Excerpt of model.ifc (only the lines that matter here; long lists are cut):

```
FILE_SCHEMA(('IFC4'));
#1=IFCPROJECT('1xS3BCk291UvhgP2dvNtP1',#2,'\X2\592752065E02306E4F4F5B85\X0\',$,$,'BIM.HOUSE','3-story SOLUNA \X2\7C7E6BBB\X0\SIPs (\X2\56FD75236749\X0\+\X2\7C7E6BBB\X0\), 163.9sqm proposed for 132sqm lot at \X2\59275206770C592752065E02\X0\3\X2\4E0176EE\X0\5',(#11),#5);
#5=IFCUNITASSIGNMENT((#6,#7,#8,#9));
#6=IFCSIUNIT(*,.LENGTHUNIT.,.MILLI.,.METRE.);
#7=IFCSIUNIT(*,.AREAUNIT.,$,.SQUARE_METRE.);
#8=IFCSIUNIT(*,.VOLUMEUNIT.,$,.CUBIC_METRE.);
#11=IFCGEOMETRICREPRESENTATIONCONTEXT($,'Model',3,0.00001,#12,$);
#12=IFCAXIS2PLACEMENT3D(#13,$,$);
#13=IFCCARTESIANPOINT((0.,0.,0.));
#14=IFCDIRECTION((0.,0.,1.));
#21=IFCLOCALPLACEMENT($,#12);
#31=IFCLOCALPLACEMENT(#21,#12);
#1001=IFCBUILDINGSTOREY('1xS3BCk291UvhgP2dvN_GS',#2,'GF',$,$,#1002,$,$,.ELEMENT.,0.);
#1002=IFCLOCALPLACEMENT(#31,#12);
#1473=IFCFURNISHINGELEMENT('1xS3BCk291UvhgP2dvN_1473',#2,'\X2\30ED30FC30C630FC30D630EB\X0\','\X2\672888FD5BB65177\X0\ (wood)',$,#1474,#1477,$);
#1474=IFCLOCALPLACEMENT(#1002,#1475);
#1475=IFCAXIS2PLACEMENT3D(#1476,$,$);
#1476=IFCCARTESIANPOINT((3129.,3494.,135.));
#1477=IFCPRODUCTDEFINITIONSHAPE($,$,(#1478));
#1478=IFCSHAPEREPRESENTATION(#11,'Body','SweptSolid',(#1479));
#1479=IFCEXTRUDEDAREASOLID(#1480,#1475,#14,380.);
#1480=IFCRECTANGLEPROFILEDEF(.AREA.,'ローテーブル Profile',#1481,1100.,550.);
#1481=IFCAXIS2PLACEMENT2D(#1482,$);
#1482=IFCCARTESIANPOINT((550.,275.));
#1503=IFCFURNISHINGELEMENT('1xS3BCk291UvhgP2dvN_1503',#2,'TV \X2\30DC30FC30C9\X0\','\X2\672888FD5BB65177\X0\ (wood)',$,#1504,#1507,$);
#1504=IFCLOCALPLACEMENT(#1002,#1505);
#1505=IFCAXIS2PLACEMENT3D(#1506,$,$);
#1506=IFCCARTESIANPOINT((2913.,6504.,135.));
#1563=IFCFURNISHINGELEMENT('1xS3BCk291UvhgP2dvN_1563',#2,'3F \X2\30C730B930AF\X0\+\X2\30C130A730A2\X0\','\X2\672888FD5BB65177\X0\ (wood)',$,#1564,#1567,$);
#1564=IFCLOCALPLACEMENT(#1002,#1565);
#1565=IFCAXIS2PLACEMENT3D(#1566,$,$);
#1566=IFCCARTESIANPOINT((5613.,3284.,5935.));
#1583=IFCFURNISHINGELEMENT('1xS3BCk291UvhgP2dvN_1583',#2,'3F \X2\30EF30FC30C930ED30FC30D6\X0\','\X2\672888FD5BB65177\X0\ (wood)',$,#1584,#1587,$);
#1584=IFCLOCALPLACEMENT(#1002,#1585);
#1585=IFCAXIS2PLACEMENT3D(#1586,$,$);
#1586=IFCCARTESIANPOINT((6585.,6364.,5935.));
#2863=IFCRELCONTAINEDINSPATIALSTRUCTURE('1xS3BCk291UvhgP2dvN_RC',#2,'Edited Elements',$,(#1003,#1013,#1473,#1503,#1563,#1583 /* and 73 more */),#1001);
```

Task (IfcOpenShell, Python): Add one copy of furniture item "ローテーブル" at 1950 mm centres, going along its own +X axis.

```python
import ifcopenshell
import ifcopenshell.api.geometry
import ifcopenshell.api.root
import ifcopenshell.util.element
import ifcopenshell.util.placement
import ifcopenshell.util.unit

model = ifcopenshell.open("model.ifc")
unit_scale = ifcopenshell.util.unit.calculate_unit_scale(model)


def reuse_history(source, copy):
    """copy_class also copies each property set's owner history, people and application; keep the originals."""
    for rel in copy.IsDefinedBy:
        if rel.is_a("IfcRelDefinesByProperties") and (history := rel.RelatingPropertyDefinition.OwnerHistory):
            rel.RelatingPropertyDefinition.OwnerHistory = source.OwnerHistory
            ifcopenshell.util.element.remove_deep2(model, history)


source = model.by_guid("1xS3BCk291UvhgP2dvN_1473")
base = ifcopenshell.util.placement.get_local_placement(source.ObjectPlacement)
step = base[:3, 0] * 1.95 / unit_scale

for i in range(1, 2):
    copy = ifcopenshell.api.root.copy_class(model, product=source)
    copy.Representation = ifcopenshell.util.element.copy_deep(
        model, source.Representation, exclude=["IfcGeometricRepresentationContext", "IfcRepresentationMap"]
    )
    reuse_history(source, copy)
    matrix = base.copy()
    matrix[:3, 3] += i * step
    print("added at", matrix[:3, 3].round(3) + 0.0)
    ifcopenshell.api.geometry.edit_object_placement(model, product=copy, matrix=matrix, is_si=False)

model.write("model_updated.ifc")
```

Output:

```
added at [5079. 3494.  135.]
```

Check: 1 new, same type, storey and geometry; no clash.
